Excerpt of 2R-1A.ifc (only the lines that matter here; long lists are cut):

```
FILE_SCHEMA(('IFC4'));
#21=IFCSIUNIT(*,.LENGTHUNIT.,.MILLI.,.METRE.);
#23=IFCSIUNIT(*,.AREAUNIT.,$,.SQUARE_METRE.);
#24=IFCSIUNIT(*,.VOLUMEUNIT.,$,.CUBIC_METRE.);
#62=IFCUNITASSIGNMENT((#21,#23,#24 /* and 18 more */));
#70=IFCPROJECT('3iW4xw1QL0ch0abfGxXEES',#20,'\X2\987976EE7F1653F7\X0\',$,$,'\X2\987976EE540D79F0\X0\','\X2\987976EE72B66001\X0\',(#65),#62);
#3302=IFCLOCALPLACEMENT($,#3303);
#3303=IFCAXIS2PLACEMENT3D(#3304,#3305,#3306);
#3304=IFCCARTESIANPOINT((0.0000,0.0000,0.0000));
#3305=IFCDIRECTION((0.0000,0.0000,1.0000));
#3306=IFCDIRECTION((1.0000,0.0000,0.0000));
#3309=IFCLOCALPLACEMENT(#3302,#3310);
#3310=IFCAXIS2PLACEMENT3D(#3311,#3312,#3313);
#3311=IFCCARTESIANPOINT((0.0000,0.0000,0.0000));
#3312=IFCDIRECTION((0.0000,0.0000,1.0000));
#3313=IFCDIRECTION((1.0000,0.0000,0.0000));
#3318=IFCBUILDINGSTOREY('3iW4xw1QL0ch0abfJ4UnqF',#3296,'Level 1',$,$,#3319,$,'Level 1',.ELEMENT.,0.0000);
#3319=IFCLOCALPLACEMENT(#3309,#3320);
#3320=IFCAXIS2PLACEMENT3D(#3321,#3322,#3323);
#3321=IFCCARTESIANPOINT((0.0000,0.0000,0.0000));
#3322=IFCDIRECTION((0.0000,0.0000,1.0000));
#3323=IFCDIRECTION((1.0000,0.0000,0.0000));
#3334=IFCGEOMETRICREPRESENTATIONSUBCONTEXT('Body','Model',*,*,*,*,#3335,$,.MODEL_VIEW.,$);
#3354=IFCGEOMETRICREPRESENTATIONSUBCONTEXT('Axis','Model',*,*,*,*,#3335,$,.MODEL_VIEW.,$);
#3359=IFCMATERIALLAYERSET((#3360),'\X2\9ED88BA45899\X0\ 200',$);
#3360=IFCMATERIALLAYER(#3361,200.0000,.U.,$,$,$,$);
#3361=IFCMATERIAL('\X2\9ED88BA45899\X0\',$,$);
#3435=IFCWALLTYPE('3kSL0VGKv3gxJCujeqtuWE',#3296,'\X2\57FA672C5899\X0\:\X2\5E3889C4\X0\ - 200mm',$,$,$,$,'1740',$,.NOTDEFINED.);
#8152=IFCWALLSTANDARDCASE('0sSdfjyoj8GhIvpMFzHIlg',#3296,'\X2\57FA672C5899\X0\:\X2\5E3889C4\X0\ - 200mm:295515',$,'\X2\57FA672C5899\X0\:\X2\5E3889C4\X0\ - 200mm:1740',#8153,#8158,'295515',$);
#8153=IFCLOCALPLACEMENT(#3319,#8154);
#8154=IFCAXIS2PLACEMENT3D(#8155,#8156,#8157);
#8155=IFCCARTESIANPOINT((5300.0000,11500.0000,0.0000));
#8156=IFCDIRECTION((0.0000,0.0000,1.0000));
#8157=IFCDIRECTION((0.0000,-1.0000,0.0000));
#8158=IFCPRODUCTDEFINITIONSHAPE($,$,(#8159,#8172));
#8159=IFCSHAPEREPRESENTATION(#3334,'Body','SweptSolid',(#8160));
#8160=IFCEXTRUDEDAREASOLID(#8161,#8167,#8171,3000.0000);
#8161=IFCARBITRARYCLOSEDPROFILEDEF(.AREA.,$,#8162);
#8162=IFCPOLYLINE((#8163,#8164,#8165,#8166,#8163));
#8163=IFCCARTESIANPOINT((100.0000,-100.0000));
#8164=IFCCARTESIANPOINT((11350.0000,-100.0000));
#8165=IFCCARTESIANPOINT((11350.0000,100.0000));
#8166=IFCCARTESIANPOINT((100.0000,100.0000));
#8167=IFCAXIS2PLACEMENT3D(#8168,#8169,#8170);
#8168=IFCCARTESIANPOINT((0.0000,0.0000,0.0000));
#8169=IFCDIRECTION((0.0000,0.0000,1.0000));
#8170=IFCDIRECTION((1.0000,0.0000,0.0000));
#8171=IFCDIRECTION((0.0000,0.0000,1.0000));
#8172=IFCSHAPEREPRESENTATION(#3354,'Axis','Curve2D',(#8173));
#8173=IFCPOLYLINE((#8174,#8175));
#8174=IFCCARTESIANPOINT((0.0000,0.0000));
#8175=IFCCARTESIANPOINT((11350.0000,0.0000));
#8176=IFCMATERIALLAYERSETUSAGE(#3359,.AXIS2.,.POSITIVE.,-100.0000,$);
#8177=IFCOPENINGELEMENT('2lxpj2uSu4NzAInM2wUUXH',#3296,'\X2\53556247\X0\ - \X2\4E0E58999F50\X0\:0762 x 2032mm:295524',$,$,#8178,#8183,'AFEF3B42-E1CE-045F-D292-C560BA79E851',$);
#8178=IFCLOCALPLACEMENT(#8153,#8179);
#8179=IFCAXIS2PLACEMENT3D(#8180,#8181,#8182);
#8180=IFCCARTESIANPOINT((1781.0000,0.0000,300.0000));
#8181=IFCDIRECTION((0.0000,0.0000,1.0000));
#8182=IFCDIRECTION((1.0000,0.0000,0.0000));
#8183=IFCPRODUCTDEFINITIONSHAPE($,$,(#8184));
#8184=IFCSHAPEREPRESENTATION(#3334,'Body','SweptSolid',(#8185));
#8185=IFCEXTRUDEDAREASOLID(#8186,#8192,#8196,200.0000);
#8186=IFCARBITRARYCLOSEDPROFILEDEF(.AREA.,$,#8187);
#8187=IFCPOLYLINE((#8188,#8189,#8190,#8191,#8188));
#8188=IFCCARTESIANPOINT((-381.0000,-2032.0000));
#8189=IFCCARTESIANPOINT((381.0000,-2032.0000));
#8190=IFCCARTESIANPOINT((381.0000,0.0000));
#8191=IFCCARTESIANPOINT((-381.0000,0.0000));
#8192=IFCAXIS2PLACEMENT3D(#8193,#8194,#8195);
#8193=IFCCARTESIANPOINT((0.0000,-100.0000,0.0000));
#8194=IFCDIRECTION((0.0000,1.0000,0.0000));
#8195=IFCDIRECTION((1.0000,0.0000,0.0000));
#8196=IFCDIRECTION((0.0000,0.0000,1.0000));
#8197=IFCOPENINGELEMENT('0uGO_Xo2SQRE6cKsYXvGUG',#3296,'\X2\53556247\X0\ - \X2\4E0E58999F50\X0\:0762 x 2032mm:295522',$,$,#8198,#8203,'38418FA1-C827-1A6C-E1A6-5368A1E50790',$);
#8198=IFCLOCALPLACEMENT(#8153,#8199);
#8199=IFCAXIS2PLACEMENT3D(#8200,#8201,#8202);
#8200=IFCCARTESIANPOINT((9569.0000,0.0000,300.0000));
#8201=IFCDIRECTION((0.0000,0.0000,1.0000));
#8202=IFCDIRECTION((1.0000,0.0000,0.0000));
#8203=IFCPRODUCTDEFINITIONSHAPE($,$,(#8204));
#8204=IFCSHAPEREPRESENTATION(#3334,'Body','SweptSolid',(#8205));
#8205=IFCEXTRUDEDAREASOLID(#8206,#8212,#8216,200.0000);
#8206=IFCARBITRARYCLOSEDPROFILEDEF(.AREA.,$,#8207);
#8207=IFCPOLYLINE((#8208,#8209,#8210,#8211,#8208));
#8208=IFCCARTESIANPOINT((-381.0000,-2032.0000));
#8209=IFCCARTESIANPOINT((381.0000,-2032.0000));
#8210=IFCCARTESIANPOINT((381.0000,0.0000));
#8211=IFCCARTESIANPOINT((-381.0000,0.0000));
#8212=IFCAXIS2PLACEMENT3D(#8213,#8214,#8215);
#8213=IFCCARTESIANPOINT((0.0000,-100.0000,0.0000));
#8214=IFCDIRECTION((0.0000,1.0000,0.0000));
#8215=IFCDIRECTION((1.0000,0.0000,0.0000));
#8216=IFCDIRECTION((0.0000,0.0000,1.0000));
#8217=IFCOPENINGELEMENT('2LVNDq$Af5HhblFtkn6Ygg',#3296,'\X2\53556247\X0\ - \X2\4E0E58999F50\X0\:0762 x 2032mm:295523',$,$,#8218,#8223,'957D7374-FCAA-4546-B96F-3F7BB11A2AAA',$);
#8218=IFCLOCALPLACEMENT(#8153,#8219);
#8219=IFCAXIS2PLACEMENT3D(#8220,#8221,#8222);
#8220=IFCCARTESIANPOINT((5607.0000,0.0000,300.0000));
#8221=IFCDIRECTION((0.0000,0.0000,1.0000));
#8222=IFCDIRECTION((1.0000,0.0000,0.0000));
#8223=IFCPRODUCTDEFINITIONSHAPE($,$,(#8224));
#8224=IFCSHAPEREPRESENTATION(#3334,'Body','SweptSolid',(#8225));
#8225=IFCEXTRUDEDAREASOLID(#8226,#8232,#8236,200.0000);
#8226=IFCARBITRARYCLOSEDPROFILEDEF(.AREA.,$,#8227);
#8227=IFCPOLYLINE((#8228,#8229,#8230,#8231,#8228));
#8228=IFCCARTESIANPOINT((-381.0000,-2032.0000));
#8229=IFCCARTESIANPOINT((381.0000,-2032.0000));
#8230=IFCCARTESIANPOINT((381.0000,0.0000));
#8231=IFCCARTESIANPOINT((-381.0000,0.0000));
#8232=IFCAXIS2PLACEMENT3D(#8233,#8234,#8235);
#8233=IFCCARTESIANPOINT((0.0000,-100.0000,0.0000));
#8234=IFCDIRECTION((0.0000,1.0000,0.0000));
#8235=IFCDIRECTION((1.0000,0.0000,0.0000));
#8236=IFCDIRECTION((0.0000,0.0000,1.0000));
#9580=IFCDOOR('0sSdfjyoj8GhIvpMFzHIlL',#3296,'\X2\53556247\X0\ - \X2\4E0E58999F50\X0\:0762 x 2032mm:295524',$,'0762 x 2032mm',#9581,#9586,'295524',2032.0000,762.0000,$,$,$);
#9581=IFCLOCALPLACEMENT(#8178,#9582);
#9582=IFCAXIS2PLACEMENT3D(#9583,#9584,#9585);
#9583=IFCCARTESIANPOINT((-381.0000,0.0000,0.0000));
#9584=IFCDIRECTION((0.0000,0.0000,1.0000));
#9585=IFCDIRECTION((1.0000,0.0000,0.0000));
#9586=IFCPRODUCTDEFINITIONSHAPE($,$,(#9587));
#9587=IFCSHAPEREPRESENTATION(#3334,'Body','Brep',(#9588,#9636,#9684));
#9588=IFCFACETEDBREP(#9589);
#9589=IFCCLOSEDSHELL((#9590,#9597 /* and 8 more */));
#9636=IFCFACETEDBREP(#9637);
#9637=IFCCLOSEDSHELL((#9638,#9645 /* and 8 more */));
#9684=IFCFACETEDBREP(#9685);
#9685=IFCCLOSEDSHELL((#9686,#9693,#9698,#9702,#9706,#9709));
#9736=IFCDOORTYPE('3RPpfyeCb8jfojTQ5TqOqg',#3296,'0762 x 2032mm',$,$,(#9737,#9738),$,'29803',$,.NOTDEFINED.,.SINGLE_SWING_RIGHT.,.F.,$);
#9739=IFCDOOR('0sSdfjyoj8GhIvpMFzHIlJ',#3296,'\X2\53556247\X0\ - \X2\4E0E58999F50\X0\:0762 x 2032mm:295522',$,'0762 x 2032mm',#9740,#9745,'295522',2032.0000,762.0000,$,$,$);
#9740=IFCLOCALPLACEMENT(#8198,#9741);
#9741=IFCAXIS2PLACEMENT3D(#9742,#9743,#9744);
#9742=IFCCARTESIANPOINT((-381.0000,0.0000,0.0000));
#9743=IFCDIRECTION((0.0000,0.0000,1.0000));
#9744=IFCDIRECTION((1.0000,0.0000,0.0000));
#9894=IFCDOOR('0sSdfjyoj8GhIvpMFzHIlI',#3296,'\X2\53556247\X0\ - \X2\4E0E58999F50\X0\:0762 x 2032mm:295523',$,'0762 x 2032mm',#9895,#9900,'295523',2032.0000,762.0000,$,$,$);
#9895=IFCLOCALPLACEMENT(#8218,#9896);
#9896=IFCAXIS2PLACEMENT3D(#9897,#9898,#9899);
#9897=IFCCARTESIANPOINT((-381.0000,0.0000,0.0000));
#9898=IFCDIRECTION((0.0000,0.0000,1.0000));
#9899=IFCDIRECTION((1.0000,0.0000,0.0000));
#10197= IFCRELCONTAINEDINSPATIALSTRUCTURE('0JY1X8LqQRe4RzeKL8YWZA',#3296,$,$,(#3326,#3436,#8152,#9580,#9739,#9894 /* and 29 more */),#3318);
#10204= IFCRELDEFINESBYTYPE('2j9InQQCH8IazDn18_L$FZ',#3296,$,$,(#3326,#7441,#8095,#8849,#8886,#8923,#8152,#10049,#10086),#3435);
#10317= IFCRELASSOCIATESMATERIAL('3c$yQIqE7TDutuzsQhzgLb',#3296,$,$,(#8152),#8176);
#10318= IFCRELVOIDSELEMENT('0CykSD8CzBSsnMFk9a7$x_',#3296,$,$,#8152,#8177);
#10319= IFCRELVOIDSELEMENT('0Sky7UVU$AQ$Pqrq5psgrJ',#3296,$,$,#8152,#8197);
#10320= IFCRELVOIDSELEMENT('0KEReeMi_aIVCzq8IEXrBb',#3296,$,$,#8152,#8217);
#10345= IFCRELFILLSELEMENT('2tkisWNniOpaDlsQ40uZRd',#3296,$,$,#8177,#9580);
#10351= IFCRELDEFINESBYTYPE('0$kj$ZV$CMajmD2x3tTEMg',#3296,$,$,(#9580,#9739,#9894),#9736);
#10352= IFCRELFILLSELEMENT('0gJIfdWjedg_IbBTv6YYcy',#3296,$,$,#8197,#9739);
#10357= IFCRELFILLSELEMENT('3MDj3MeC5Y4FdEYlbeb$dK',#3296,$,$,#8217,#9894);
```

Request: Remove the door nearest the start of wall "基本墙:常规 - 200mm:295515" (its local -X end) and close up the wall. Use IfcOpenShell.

```python
import ifcopenshell
import ifcopenshell.api.feature
import ifcopenshell.api.root
import ifcopenshell.geom
import ifcopenshell.util.shape

model = ifcopenshell.open("2R-1A.ifc")
settings = ifcopenshell.geom.settings()


def volume(element):
    """Net volume in cubic metres, openings subtracted."""
    shape = ifcopenshell.geom.create_shape(settings, element)
    return ifcopenshell.util.shape.get_volume(shape.geometry)


door = model.by_id(9580)
opening = door.FillsVoids[0].RelatingOpeningElement
wall = opening.VoidsElements[0].RelatingBuildingElement
before = volume(wall)

ifcopenshell.api.root.remove_product(model, product=door)
ifcopenshell.api.feature.remove_feature(model, feature=opening)

after = volume(wall)

print(f"wall volume {before:.3f} -> {after:.3f} m3")

model.write("2R-1A_updated.ifc")
```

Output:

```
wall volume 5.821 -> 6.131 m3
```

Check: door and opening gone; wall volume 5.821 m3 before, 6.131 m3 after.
